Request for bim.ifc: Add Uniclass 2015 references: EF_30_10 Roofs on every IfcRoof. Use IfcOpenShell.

First a look at what the model holds.

```python
import ifcopenshell

model = ifcopenshell.open("bim.ifc")
print(model.schema)
print("classifications:", [c.Name for c in model.by_type("IfcClassification")])
for ifc_class in ("IfcDoor", "IfcRoof", "IfcStair", "IfcWall", "IfcWindow"):
    print(ifc_class, len(model.by_type(ifc_class)))
```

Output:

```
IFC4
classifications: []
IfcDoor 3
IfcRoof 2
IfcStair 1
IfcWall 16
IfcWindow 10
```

```python
import ifcopenshell
import ifcopenshell.api.classification

model = ifcopenshell.open("bim.ifc")

system = ifcopenshell.api.classification.add_classification(model, classification="Uniclass 2015")

codes = {
    "IfcRoof": ("EF_30_10", "Roofs"),
}
for ifc_class, (code, name) in codes.items():
    products = model.by_type(ifc_class)
    ifcopenshell.api.classification.add_reference(
        model, products=products, classification=system, identification=code, name=name
    )
    print(code, len(products))

model.write("bim_v2.ifc")
```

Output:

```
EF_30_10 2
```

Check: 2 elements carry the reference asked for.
